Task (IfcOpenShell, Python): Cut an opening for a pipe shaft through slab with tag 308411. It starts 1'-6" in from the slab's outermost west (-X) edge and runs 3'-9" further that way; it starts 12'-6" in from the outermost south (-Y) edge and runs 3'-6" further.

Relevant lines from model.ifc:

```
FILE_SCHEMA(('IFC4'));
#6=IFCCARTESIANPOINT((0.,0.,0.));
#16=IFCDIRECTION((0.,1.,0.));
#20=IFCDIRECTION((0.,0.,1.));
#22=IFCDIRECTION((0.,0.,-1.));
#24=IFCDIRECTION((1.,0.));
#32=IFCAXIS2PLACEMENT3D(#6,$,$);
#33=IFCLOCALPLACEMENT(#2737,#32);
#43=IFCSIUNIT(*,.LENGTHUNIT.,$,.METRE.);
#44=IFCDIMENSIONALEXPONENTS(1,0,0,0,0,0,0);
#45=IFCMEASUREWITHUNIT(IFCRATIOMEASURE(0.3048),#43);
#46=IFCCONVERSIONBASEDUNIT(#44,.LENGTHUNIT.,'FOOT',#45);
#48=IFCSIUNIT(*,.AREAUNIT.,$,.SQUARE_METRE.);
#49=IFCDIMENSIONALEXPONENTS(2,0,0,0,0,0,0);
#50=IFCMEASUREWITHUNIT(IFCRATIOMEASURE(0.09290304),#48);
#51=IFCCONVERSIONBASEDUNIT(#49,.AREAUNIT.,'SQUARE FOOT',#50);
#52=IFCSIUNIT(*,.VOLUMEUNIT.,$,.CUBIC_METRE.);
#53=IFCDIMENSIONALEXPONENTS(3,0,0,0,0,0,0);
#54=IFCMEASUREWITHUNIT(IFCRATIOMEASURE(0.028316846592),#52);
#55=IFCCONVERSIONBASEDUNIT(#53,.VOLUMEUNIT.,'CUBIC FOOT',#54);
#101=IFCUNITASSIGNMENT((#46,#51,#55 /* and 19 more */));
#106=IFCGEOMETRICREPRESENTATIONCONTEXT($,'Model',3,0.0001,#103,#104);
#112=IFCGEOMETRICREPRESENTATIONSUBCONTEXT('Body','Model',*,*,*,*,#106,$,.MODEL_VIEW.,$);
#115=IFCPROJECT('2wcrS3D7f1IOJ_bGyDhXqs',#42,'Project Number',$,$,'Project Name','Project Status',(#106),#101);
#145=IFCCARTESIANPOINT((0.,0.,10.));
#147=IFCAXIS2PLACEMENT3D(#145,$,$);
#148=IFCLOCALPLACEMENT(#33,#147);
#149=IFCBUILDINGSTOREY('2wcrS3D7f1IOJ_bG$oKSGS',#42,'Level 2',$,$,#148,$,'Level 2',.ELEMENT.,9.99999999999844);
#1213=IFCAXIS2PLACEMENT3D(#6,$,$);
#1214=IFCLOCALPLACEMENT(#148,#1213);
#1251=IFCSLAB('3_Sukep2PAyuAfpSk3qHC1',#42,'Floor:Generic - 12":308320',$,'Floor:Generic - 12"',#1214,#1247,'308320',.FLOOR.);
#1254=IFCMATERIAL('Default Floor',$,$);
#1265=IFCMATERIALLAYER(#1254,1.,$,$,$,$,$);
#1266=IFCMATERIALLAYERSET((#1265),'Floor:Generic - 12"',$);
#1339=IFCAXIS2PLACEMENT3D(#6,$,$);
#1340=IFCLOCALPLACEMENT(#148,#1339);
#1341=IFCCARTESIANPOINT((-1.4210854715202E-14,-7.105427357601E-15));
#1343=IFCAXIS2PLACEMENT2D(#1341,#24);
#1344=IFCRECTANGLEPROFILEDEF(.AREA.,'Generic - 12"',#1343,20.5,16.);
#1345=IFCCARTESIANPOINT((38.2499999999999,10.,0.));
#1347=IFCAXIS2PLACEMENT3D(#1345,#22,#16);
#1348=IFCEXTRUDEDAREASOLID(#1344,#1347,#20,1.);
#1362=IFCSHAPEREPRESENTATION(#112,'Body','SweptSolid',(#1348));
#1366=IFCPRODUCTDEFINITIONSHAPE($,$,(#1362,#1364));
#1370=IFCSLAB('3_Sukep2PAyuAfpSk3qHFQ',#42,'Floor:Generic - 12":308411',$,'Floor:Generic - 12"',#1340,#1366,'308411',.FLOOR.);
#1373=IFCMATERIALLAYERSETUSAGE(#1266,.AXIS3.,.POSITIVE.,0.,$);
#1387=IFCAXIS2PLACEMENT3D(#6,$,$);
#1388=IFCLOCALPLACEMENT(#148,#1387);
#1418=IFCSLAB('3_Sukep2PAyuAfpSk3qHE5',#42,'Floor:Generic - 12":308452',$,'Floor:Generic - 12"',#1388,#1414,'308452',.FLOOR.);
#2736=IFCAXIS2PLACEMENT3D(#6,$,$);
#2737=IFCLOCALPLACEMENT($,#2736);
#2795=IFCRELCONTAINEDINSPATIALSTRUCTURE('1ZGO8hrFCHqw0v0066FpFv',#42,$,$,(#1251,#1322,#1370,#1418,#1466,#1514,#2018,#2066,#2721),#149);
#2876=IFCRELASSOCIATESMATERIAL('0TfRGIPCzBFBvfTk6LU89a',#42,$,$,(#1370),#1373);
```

```python
import numpy as np
import ifcopenshell
import ifcopenshell.api.feature
import ifcopenshell.api.geometry
import ifcopenshell.api.root
import ifcopenshell.geom
import ifcopenshell.util.placement
import ifcopenshell.util.representation
import ifcopenshell.util.shape
import ifcopenshell.util.unit

model = ifcopenshell.open("model.ifc")
unit_scale = ifcopenshell.util.unit.calculate_unit_scale(model)
settings = ifcopenshell.geom.settings()


def volume(element):
    """Net volume in cubic metres, openings subtracted."""
    shape = ifcopenshell.geom.create_shape(settings, element)
    return ifcopenshell.util.shape.get_volume(shape.geometry)


slab = model.by_guid("3_Sukep2PAyuAfpSk3qHFQ")
before = volume(slab)

# Extent in the slab's own axes, in metres. The edges named are its -X and -Y sides.
slab_shape = ifcopenshell.geom.create_shape(settings, slab)
vertices = ifcopenshell.util.shape.get_vertices(slab_shape.geometry)
x_min, y_min, bottom = vertices.min(axis=0)
top = vertices[:, 2].max()

opening = ifcopenshell.api.root.create_entity(model, ifc_class="IfcOpeningElement", name="Pipe shaft opening", predefined_type="OPENING")
context = ifcopenshell.util.representation.get_context(model, "Model", "Body", "MODEL_VIEW")
width, depth = 1.143, 1.0668
outline = [(0.0, 0.0), (width, 0.0), (width, depth), (0.0, depth), (0.0, 0.0)]
# Overshoot both faces by 50 mm so the cut is clean.
shape = ifcopenshell.api.geometry.add_slab_representation(
    model, context=context, depth=top - bottom + 0.1, polyline=outline
)
ifcopenshell.api.geometry.assign_representation(model, product=opening, representation=shape)

matrix = ifcopenshell.util.placement.get_local_placement(slab.ObjectPlacement)
matrix[:, 3] = matrix @ np.append(np.array([x_min + 0.4572, y_min + 3.81, bottom - 0.05]) / unit_scale, 1.0)
ifcopenshell.api.geometry.edit_object_placement(model, product=opening, matrix=matrix, is_si=False)
ifcopenshell.api.feature.add_feature(model, feature=opening, element=slab)

after = volume(slab)

print(f"slab volume {before:.3f} -> {after:.3f} m3")

model.write("model-out.ifc")
```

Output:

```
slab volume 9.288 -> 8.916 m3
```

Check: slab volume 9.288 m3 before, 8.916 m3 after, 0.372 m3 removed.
